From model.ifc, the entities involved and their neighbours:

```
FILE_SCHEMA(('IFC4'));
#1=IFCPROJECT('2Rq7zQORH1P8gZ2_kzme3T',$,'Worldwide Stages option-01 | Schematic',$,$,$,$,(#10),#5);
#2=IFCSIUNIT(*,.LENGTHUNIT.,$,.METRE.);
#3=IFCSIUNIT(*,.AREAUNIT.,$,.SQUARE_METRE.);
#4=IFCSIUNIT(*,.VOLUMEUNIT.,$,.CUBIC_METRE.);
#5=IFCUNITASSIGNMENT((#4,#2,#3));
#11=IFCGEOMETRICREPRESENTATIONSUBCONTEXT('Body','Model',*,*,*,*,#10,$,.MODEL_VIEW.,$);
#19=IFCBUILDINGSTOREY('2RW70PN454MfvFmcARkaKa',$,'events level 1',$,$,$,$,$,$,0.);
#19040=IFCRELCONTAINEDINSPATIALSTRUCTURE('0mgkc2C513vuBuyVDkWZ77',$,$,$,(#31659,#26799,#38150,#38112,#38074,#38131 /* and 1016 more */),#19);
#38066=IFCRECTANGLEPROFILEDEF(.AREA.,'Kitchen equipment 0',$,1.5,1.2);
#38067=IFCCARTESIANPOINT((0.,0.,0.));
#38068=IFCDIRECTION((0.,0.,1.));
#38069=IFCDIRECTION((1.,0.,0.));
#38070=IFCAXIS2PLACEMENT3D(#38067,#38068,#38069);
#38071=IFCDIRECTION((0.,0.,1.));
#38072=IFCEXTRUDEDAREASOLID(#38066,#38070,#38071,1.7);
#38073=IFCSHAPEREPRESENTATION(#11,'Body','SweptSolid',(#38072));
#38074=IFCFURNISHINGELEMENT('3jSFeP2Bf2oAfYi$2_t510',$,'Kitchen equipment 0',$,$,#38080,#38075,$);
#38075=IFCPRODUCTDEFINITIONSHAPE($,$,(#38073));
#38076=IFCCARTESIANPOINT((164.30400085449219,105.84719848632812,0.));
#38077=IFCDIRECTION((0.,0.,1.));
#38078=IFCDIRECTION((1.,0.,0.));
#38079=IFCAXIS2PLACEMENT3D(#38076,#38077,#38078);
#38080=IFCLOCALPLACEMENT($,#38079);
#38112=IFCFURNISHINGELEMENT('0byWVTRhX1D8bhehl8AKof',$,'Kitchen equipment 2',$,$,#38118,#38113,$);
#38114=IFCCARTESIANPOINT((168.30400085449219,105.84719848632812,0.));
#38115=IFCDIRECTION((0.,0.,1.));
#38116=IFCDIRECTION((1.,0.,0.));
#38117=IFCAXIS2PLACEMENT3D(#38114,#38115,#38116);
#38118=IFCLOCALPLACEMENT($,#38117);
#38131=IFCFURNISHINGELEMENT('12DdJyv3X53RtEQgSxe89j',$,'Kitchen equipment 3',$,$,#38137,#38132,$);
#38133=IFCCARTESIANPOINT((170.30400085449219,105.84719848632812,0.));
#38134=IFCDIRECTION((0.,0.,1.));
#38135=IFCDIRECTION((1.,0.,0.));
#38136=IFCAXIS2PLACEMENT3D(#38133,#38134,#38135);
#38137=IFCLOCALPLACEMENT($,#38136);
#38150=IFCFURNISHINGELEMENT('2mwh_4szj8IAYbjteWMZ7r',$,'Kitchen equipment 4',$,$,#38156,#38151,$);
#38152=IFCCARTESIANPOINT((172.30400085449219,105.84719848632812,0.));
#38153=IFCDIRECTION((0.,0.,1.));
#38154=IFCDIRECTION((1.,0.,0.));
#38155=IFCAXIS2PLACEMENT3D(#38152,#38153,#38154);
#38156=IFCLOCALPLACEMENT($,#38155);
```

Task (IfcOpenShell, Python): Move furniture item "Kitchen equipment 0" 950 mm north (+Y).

```python
import ifcopenshell
import ifcopenshell.api.geometry
import ifcopenshell.util.placement
import ifcopenshell.util.unit

model = ifcopenshell.open("model.ifc")
unit_scale = ifcopenshell.util.unit.calculate_unit_scale(model)

item = model.by_guid("3jSFeP2Bf2oAfYi$2_t510")
matrix = ifcopenshell.util.placement.get_local_placement(item.ObjectPlacement)
matrix[1, 3] += 0.95 / unit_scale
ifcopenshell.api.geometry.edit_object_placement(model, product=item, matrix=matrix, is_si=False)

print(ifcopenshell.util.placement.get_local_placement(item.ObjectPlacement).round(3) + 0.0)

model.write("model-out.ifc")
```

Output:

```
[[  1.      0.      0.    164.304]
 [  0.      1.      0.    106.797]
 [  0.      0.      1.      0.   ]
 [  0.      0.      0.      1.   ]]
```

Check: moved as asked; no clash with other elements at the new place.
